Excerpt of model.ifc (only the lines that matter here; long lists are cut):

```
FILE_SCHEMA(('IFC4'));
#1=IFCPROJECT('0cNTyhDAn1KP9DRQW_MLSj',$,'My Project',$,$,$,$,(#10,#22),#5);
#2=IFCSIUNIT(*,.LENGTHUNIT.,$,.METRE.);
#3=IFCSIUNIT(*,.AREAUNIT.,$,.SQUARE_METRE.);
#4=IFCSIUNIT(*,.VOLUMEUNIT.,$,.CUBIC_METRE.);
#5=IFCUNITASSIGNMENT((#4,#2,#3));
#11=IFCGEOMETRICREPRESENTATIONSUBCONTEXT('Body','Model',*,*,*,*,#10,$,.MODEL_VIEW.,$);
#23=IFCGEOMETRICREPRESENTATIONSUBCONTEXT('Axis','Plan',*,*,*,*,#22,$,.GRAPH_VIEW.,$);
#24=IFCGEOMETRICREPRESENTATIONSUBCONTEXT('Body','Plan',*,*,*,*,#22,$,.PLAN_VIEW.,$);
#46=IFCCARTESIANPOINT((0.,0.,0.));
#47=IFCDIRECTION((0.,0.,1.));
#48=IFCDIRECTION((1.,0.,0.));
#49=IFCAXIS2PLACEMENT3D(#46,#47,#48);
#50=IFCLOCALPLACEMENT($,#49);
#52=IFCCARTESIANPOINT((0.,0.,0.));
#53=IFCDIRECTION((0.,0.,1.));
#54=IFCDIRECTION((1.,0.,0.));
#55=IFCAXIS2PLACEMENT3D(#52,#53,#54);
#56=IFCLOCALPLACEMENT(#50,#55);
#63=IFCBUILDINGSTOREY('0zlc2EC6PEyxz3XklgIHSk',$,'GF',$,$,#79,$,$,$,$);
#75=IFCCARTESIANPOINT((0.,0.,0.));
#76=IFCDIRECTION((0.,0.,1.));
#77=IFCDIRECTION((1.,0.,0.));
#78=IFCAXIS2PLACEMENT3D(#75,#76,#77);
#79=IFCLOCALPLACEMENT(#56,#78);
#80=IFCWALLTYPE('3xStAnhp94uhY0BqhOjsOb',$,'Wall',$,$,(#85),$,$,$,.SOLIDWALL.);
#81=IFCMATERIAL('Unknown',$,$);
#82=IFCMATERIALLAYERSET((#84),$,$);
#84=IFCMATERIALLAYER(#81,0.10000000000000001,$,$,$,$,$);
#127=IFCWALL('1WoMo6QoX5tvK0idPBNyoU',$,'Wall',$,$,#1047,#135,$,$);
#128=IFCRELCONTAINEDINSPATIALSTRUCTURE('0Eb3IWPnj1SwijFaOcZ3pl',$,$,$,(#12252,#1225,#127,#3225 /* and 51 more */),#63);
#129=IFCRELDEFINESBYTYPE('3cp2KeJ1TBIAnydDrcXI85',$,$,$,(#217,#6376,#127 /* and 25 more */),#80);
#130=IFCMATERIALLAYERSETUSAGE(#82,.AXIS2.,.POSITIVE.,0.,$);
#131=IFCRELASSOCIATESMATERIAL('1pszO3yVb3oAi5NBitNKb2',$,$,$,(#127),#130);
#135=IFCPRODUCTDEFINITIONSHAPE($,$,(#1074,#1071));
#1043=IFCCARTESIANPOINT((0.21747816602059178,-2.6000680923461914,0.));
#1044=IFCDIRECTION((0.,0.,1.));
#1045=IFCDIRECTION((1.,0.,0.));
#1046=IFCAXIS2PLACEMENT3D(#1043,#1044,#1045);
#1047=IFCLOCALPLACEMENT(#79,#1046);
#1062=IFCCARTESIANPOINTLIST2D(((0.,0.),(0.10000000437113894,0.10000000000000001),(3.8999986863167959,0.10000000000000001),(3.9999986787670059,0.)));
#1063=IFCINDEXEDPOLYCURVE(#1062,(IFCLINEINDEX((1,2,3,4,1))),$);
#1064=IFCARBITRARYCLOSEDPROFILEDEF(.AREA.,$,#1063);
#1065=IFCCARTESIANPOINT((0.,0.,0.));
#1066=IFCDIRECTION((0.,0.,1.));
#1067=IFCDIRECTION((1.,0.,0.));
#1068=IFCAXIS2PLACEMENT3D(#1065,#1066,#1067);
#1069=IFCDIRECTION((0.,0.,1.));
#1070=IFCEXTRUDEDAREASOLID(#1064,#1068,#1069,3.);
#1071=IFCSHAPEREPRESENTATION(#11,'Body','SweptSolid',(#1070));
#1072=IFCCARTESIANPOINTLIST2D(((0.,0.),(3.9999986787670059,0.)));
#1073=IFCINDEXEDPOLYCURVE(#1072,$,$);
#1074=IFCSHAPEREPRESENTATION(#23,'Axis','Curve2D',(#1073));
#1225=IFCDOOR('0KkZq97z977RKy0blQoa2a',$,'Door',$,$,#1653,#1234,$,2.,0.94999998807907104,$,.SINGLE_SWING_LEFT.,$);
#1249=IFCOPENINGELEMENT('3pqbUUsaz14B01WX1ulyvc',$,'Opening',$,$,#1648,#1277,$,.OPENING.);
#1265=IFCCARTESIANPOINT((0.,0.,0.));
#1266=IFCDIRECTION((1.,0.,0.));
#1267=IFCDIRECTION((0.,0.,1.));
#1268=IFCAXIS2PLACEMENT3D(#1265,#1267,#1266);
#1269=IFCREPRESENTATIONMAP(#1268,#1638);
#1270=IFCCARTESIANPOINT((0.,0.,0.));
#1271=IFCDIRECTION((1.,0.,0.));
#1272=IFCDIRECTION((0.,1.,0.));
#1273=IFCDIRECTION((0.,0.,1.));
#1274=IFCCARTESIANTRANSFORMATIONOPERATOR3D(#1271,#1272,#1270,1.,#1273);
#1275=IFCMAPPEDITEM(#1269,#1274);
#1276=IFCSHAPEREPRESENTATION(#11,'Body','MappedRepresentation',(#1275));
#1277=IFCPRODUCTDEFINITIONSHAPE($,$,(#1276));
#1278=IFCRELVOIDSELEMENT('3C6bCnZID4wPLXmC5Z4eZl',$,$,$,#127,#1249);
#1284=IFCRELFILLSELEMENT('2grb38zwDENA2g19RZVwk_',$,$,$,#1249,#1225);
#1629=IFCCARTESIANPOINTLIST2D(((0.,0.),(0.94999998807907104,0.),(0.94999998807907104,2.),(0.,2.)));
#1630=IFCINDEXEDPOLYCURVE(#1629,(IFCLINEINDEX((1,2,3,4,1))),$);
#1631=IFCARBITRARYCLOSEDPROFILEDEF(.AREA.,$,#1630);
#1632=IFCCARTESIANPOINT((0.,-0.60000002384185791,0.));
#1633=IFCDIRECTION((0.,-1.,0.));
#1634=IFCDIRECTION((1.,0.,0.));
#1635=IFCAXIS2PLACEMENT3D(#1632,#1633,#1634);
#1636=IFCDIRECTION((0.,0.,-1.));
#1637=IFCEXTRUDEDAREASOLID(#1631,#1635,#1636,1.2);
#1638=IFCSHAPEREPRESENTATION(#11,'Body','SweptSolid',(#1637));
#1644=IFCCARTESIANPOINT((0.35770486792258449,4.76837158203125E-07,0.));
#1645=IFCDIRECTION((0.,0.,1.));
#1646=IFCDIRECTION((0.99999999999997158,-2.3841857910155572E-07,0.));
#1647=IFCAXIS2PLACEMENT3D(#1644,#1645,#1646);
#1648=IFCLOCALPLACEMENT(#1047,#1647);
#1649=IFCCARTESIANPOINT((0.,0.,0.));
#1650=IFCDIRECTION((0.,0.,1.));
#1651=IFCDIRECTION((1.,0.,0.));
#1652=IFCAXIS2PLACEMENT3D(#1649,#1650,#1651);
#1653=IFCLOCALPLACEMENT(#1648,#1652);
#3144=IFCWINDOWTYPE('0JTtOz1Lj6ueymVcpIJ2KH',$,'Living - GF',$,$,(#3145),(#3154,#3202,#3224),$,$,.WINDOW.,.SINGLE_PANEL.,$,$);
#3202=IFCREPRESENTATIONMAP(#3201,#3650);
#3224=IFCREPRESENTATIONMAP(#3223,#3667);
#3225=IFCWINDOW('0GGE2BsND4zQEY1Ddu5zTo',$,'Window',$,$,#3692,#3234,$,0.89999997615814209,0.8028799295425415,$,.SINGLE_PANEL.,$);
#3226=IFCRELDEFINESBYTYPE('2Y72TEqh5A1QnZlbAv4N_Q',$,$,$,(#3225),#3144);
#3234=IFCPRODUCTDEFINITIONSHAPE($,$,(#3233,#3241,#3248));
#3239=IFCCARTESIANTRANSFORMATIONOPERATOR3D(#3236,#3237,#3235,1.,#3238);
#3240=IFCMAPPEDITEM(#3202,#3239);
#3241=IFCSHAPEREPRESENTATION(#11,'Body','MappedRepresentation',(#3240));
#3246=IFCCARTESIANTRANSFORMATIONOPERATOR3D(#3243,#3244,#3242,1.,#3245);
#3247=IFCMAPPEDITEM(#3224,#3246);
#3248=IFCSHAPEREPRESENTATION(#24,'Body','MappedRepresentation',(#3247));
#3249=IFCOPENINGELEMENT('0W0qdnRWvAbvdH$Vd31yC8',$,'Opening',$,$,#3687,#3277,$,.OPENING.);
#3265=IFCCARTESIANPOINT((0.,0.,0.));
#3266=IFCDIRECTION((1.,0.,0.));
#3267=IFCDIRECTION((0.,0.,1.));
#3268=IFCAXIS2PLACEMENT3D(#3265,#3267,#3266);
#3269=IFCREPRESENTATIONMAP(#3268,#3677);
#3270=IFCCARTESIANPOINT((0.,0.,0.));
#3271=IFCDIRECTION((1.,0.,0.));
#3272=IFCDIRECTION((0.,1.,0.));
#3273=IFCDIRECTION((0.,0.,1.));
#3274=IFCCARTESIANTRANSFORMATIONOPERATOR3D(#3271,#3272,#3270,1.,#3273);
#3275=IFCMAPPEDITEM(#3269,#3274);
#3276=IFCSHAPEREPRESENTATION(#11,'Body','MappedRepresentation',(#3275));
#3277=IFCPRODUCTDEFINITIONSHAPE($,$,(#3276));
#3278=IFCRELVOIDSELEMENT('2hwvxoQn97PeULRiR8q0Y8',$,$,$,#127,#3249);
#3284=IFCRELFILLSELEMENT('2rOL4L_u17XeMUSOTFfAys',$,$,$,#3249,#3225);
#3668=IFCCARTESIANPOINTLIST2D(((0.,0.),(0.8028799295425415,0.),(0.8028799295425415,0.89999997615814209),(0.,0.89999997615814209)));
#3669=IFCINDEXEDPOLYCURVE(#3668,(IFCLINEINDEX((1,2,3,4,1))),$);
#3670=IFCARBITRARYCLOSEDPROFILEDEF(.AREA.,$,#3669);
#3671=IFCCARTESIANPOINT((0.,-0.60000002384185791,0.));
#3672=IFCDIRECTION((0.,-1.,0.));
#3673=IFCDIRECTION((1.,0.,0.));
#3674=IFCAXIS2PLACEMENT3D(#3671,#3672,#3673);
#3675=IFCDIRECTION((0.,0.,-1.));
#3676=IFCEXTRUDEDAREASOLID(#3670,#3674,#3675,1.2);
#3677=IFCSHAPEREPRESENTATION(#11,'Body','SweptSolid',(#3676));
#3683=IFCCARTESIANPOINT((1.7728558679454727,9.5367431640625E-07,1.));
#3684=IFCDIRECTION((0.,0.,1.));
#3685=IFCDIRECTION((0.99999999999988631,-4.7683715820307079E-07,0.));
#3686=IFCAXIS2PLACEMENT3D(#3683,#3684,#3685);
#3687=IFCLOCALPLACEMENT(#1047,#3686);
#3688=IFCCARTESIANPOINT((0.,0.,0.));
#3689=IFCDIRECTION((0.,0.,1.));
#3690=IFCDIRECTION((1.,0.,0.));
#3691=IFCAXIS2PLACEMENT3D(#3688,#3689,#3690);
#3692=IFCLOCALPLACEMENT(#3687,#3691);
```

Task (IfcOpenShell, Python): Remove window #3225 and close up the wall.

```python
import ifcopenshell
import ifcopenshell.api.feature
import ifcopenshell.api.root
import ifcopenshell.geom
import ifcopenshell.util.shape

model = ifcopenshell.open("model.ifc")
settings = ifcopenshell.geom.settings()


def volume(element):
    """Net volume in cubic metres, openings subtracted."""
    shape = ifcopenshell.geom.create_shape(settings, element)
    return ifcopenshell.util.shape.get_volume(shape.geometry)


window = model.by_guid("0GGE2BsND4zQEY1Ddu5zTo")
opening = window.FillsVoids[0].RelatingOpeningElement
wall = opening.VoidsElements[0].RelatingBuildingElement
before = volume(wall)

ifcopenshell.api.root.remove_product(model, product=window)
ifcopenshell.api.feature.remove_feature(model, feature=opening)

after = volume(wall)

print(f"wall volume {before:.3f} -> {after:.3f} m3")

model.write("model-out.ifc")
```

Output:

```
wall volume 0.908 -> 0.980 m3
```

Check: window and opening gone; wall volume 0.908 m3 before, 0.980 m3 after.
